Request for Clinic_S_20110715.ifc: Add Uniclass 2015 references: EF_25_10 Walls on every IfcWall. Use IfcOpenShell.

First a look at what the model holds.

```python
import ifcopenshell

model = ifcopenshell.open("Clinic_S_20110715.ifc")
print(model.schema)
print("classifications:", [c.Name for c in model.by_type("IfcClassification")])
for ifc_class in ("IfcDoor", "IfcRoof", "IfcStair", "IfcWall", "IfcWindow"):
    print(ifc_class, len(model.by_type(ifc_class)))
```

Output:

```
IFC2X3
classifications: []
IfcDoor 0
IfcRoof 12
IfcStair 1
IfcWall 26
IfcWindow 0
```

```python
import ifcopenshell
import ifcopenshell.api.classification

model = ifcopenshell.open("Clinic_S_20110715.ifc")

# IFC2X3 requires Source and Edition and has no link from the project to the system.
system = model.create_entity("IfcClassification", Source="NBS", Edition="2015", Name="Uniclass 2015")

codes = {
    "IfcWall": ("EF_25_10", "Walls"),
}
for ifc_class, (code, name) in codes.items():
    products = model.by_type(ifc_class)
    ifcopenshell.api.classification.add_reference(
        model, products=products, classification=system, identification=code, name=name
    )
    print(code, len(products))

model.write("Clinic_S_20110715_rev.ifc")
```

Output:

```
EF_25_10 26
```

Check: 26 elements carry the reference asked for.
